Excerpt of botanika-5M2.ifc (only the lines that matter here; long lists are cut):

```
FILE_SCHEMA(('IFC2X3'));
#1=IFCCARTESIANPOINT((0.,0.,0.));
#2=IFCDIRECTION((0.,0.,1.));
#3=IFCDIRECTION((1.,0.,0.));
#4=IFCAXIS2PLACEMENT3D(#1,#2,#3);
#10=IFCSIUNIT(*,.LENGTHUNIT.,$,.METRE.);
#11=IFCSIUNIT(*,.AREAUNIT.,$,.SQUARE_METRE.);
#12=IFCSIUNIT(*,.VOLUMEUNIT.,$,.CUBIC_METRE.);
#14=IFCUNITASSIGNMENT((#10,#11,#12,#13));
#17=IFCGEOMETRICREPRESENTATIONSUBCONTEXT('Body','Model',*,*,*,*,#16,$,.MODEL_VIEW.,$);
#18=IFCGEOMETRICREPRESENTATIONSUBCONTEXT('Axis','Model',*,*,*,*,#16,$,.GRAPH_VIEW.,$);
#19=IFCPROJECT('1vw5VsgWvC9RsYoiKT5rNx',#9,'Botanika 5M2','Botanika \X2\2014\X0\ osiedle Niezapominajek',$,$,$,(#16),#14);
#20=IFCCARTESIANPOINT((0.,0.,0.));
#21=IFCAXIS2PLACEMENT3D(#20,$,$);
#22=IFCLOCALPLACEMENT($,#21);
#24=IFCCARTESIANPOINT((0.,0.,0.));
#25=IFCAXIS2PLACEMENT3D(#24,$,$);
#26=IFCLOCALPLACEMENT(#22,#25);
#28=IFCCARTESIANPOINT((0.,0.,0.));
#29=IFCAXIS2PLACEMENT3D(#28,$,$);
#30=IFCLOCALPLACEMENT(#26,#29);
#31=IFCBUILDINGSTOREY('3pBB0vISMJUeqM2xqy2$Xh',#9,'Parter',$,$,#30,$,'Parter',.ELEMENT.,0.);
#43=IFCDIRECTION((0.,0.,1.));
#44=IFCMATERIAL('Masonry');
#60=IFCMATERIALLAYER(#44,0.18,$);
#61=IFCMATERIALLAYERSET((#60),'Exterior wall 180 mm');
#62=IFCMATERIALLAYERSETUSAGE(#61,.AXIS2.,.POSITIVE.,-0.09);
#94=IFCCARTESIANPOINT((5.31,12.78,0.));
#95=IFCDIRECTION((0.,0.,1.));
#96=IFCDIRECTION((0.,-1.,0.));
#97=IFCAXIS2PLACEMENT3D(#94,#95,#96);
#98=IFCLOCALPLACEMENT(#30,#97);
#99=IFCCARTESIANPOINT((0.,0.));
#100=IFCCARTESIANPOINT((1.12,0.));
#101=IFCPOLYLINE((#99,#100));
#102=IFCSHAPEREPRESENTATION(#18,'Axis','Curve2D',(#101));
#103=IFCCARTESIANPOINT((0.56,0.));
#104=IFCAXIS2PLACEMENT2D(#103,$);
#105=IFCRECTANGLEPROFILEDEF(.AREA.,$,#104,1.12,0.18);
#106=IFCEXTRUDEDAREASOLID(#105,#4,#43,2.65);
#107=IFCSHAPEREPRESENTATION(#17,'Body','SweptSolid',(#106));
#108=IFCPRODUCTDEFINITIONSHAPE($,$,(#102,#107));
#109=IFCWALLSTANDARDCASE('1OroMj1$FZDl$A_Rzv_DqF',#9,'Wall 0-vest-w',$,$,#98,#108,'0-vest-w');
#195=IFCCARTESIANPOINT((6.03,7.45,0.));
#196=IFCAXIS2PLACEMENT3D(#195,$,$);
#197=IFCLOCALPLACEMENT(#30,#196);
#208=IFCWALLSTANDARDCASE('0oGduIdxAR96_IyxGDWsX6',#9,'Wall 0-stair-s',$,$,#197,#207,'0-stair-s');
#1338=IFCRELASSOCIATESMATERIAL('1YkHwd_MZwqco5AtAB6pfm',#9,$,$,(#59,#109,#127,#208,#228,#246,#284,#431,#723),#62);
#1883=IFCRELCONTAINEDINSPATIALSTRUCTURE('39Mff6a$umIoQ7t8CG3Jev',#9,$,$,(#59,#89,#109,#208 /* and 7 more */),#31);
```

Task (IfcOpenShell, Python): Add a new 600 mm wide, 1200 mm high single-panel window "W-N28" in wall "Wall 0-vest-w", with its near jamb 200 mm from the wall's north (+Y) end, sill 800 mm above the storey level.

```python
import numpy as np
import ifcopenshell
import ifcopenshell.api.feature
import ifcopenshell.api.geometry
import ifcopenshell.api.root
import ifcopenshell.api.spatial
import ifcopenshell.api.type
import ifcopenshell.geom
import ifcopenshell.util.element
import ifcopenshell.util.placement
import ifcopenshell.util.representation
import ifcopenshell.util.shape
import ifcopenshell.util.unit

model = ifcopenshell.open("botanika-5M2.ifc")
unit_scale = ifcopenshell.util.unit.calculate_unit_scale(model)
settings = ifcopenshell.geom.settings()


def volume(element):
    """Net volume in cubic metres, openings subtracted."""
    shape = ifcopenshell.geom.create_shape(settings, element)
    return ifcopenshell.util.shape.get_volume(shape.geometry)


wall = model.by_guid("1OroMj1$FZDl$A_Rzv_DqF")
storey = ifcopenshell.util.element.get_container(wall, ifc_class="IfcBuildingStorey")
context = ifcopenshell.util.representation.get_context(model, "Model", "Body", "MODEL_VIEW")
before = volume(wall)

width, height, from_end, sill = 0.6, 1.2, 0.2, 0.8  # metres

# The wall runs along its own X axis, and the end named is its -X end.
wall_shape = ifcopenshell.geom.create_shape(settings, wall)
x, y, z = ifcopenshell.util.shape.get_vertices(wall_shape.geometry).T
start = x.min() + from_end
face, thickness = float(y.min()), float(y.max() - y.min())
wall_matrix = ifcopenshell.util.placement.get_local_placement(wall.ObjectPlacement)
level = ifcopenshell.util.placement.get_local_placement(storey.ObjectPlacement)[2, 3]


def in_wall(x, y):
    """Placement at x, y metres in the wall's axes, at sill height."""
    matrix = wall_matrix.copy()
    matrix[:, 3] = wall_matrix @ np.array([x / unit_scale, y / unit_scale, 0.0, 1.0])
    matrix[2, 3] = level + sill / unit_scale
    return matrix


# Opening: a box that overshoots both wall faces by 50 mm.
opening = ifcopenshell.api.root.create_entity(model, ifc_class="IfcOpeningElement")
box = ifcopenshell.api.geometry.add_wall_representation(
    model, context=context, length=width, height=height, thickness=thickness + 0.1
)
ifcopenshell.api.geometry.assign_representation(model, product=opening, representation=box)
ifcopenshell.api.geometry.edit_object_placement(model, product=opening, matrix=in_wall(start, face - 0.05), is_si=False)
ifcopenshell.api.feature.add_feature(model, feature=opening, element=wall)

window = ifcopenshell.api.root.create_entity(model, ifc_class="IfcWindow", name="W-N28")
window.OverallWidth, window.OverallHeight = width / unit_scale, height / unit_scale
body = ifcopenshell.api.geometry.add_window_representation(
    model,
    context=context,
    overall_width=window.OverallWidth,
    overall_height=window.OverallHeight,
    partition_type="SINGLE_PANEL",
)
ifcopenshell.api.geometry.assign_representation(model, product=window, representation=body)
ifcopenshell.api.spatial.assign_container(model, products=[window], relating_structure=storey)
fills = ifcopenshell.api.feature.add_filling(model, opening=opening, element=window)
fills.OwnerHistory = window.OwnerHistory  # required in IFC2X3

# IFC2X3 keeps the operation on the window style.
style = ifcopenshell.api.root.create_entity(model, ifc_class="IfcWindowStyle", name="W-N28")
style.OperationType, style.ConstructionType = "SINGLE_PANEL", "NOTDEFINED"
style.ParameterTakesPrecedence = style.Sizeable = False
ifcopenshell.api.type.assign_type(model, related_objects=[window], relating_type=style)

# Centre the window in the wall's thickness.
ifcopenshell.api.geometry.edit_object_placement(model, product=window, matrix=in_wall(start, face), is_si=False)
window_shape = ifcopenshell.geom.create_shape(settings, window)
depth = ifcopenshell.util.shape.get_vertices(window_shape.geometry)[:, 1]
offset = face + thickness / 2 - (depth.min() + depth.max()) / 2
ifcopenshell.api.geometry.edit_object_placement(model, product=window, matrix=in_wall(start, offset), is_si=False)

after = volume(wall)

print(f"wall volume {before:.3f} -> {after:.3f} m3")

model.write("botanika-5M2_edited.ifc")
```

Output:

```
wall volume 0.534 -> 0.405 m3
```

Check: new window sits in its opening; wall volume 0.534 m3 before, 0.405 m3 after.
